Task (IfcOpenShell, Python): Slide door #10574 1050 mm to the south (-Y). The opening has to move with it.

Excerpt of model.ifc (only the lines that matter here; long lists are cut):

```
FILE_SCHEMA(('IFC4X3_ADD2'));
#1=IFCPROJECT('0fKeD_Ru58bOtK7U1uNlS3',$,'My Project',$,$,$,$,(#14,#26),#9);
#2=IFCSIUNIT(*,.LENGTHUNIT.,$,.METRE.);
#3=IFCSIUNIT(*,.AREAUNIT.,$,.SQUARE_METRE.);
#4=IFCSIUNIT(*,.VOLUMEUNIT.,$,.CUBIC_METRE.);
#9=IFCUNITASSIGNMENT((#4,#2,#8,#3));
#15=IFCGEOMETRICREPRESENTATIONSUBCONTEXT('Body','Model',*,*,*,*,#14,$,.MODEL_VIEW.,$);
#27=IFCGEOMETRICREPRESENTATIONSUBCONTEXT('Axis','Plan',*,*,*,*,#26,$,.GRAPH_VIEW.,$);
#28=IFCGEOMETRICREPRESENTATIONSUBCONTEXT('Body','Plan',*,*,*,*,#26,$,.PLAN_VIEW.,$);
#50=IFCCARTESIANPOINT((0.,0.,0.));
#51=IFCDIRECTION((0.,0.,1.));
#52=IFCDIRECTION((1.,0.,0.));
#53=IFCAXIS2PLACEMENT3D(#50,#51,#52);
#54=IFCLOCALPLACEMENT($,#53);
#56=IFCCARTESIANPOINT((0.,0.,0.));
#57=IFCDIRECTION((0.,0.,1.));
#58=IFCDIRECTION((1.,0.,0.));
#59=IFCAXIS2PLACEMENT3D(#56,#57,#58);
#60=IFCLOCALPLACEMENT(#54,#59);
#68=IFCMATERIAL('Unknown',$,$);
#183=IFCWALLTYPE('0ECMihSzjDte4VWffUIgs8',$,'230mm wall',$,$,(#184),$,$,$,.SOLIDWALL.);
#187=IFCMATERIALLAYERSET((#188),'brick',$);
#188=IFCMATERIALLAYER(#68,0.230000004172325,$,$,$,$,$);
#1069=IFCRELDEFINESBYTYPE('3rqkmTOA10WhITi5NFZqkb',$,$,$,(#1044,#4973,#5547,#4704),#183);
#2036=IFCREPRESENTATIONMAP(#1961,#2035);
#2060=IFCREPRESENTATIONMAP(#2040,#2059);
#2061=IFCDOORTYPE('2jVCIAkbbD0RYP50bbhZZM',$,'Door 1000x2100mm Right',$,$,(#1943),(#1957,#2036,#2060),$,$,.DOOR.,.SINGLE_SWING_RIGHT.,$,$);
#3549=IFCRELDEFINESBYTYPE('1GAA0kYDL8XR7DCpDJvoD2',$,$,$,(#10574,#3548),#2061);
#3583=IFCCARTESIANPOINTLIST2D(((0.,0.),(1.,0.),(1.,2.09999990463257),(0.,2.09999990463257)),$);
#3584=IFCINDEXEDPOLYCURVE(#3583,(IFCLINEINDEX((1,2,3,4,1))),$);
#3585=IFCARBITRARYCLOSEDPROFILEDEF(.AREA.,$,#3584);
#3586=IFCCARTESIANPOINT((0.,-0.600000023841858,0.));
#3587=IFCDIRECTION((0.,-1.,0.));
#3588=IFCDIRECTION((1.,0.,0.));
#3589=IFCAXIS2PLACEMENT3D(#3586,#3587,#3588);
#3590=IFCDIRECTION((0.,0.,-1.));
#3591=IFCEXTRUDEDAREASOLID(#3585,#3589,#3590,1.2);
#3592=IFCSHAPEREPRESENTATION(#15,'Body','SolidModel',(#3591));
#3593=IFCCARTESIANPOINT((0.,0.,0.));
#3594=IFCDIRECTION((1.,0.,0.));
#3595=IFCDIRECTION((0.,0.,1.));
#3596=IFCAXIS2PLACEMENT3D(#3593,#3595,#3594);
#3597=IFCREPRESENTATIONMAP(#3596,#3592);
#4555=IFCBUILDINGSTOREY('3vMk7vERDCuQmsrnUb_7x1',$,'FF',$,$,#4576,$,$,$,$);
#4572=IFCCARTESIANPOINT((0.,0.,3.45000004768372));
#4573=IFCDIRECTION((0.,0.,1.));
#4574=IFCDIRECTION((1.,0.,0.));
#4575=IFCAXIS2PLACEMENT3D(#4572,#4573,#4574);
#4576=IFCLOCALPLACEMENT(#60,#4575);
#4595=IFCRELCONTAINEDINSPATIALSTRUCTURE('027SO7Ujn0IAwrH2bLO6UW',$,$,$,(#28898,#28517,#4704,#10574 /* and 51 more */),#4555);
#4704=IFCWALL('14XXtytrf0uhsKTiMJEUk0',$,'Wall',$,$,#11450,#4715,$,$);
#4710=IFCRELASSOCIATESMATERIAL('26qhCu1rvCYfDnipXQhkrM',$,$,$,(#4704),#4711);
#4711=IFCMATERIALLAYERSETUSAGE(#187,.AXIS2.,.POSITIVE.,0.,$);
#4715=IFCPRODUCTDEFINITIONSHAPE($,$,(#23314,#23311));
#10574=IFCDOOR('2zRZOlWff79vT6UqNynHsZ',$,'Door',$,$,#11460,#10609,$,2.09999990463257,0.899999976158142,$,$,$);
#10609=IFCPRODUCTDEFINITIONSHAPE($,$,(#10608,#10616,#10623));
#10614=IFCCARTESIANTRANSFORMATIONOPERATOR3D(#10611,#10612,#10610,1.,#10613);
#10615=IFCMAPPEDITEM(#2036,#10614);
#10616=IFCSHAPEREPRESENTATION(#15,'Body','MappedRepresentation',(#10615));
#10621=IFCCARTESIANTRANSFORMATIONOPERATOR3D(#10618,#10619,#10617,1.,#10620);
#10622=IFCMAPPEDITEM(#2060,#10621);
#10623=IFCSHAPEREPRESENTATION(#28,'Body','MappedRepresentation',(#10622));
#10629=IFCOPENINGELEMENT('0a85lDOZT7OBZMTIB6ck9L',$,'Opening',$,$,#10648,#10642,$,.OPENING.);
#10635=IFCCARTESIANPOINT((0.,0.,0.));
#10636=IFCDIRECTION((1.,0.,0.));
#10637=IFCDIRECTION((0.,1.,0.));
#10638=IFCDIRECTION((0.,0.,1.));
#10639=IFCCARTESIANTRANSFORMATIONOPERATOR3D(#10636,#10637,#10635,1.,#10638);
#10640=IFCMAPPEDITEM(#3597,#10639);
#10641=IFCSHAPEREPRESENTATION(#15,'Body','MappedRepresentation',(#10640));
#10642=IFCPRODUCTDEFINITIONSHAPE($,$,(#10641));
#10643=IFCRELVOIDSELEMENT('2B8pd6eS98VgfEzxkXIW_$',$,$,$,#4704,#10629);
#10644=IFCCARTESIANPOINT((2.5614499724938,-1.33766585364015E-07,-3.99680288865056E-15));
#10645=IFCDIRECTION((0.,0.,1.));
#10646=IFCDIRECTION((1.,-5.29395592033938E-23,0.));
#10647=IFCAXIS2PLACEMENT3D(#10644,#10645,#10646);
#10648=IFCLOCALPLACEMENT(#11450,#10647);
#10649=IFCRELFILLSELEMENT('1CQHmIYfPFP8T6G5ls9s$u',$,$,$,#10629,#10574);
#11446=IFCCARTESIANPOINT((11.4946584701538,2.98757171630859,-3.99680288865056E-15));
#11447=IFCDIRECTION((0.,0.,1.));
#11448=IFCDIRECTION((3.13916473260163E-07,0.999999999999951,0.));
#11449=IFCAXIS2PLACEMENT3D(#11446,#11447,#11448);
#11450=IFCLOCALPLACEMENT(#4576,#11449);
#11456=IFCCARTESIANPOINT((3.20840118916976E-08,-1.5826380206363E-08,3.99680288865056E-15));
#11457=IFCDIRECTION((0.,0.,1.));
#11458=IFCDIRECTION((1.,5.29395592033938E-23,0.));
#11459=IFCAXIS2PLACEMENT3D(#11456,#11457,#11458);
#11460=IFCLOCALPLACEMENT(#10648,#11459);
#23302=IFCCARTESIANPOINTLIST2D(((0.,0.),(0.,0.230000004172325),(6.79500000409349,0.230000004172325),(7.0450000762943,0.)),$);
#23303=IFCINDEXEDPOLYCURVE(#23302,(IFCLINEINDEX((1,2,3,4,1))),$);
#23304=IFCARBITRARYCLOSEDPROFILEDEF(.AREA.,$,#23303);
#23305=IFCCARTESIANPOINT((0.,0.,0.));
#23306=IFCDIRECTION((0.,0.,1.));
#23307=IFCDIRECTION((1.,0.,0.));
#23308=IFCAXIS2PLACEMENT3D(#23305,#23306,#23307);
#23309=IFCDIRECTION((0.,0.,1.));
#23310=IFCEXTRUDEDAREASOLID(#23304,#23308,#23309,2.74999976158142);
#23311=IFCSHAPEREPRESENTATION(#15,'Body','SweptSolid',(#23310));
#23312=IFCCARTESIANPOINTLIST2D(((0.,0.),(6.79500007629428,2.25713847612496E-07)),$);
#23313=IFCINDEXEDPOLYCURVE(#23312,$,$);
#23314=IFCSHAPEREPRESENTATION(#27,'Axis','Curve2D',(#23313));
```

```python
import ifcopenshell
import ifcopenshell.api.geometry
import ifcopenshell.util.placement
import ifcopenshell.util.unit

model = ifcopenshell.open("model.ifc")
unit_scale = ifcopenshell.util.unit.calculate_unit_scale(model)

door = model.by_id(10574)
opening = door.FillsVoids[0].RelatingOpeningElement
wall = opening.VoidsElements[0].RelatingBuildingElement

wall_matrix = ifcopenshell.util.placement.get_local_placement(wall.ObjectPlacement)
shift = wall_matrix[:3, 0] * -1.05 / unit_scale
before = ifcopenshell.util.placement.get_local_placement(door.ObjectPlacement)[:3, 3].copy()

# The door is placed relative to its opening, so it follows when the opening moves.
matrix = ifcopenshell.util.placement.get_local_placement(opening.ObjectPlacement)
matrix[:3, 3] += shift
ifcopenshell.api.geometry.edit_object_placement(
    model, product=opening, matrix=matrix, is_si=False, should_transform_children=True
)

after = ifcopenshell.util.placement.get_local_placement(door.ObjectPlacement)[:3, 3]
print("door moved by", (after - before).round(3) + 0.0)

model.write("model-out.ifc")
```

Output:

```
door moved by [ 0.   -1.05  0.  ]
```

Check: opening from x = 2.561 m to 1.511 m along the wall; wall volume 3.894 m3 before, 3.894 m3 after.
